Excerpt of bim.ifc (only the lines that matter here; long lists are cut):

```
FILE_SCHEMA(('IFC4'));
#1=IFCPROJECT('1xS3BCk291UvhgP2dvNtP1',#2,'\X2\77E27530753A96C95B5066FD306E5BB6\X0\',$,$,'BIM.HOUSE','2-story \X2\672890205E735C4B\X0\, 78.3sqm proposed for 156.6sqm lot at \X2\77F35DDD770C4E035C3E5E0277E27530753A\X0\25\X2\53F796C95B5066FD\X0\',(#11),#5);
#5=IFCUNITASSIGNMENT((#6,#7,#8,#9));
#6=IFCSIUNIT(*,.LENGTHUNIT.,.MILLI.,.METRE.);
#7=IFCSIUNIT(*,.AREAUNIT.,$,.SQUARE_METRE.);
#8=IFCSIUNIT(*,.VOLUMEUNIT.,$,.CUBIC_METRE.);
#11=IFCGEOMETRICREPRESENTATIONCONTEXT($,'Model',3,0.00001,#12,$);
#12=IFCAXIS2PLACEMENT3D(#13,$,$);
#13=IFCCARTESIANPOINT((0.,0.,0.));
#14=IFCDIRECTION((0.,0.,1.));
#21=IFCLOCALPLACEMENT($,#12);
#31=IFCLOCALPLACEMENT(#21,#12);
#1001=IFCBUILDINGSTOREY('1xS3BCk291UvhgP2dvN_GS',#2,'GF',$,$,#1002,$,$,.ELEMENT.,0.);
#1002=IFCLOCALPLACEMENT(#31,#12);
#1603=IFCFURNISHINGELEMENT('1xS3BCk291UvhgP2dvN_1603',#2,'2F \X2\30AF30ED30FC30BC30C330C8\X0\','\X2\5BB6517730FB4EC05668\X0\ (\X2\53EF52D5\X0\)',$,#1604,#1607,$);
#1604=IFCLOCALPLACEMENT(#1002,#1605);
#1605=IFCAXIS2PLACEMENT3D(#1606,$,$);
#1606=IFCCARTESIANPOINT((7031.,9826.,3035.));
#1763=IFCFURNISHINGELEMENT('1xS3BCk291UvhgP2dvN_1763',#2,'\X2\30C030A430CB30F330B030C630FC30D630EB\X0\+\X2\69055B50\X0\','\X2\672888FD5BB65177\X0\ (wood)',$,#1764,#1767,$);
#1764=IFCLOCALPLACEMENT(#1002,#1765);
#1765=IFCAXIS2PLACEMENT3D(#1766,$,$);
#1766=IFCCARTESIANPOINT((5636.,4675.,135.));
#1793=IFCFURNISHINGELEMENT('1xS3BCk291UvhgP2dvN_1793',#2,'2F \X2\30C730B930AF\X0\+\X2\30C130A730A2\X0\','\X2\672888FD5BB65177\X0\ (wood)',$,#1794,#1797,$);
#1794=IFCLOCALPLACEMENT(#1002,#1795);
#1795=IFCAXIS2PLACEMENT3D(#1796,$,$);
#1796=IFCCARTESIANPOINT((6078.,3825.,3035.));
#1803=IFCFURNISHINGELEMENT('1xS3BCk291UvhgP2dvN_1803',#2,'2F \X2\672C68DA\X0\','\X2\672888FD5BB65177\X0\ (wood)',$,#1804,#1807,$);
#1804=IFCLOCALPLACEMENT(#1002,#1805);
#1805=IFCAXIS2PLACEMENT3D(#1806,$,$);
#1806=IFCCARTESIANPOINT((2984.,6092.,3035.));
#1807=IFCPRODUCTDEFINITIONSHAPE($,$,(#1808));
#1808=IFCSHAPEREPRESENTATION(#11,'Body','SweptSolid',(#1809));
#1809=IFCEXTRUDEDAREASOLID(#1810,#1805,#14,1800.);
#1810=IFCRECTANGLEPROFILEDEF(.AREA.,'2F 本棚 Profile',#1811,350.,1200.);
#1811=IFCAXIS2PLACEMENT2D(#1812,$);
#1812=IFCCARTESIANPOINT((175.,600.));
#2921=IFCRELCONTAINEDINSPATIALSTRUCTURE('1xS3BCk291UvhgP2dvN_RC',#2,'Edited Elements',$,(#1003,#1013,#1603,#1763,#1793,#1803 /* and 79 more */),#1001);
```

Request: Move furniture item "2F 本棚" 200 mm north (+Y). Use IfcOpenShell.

```python
import ifcopenshell
import ifcopenshell.api.geometry
import ifcopenshell.util.placement
import ifcopenshell.util.unit

model = ifcopenshell.open("bim.ifc")
unit_scale = ifcopenshell.util.unit.calculate_unit_scale(model)

item = model.by_guid("1xS3BCk291UvhgP2dvN_1803")
matrix = ifcopenshell.util.placement.get_local_placement(item.ObjectPlacement)
matrix[1, 3] += 0.2 / unit_scale
ifcopenshell.api.geometry.edit_object_placement(model, product=item, matrix=matrix, is_si=False)

print(ifcopenshell.util.placement.get_local_placement(item.ObjectPlacement).round(3) + 0.0)

model.write("bim_updated.ifc")
```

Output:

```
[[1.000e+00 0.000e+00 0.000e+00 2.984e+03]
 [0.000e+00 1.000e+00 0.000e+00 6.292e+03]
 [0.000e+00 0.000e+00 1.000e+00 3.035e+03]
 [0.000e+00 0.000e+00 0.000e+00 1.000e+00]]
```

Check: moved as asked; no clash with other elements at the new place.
